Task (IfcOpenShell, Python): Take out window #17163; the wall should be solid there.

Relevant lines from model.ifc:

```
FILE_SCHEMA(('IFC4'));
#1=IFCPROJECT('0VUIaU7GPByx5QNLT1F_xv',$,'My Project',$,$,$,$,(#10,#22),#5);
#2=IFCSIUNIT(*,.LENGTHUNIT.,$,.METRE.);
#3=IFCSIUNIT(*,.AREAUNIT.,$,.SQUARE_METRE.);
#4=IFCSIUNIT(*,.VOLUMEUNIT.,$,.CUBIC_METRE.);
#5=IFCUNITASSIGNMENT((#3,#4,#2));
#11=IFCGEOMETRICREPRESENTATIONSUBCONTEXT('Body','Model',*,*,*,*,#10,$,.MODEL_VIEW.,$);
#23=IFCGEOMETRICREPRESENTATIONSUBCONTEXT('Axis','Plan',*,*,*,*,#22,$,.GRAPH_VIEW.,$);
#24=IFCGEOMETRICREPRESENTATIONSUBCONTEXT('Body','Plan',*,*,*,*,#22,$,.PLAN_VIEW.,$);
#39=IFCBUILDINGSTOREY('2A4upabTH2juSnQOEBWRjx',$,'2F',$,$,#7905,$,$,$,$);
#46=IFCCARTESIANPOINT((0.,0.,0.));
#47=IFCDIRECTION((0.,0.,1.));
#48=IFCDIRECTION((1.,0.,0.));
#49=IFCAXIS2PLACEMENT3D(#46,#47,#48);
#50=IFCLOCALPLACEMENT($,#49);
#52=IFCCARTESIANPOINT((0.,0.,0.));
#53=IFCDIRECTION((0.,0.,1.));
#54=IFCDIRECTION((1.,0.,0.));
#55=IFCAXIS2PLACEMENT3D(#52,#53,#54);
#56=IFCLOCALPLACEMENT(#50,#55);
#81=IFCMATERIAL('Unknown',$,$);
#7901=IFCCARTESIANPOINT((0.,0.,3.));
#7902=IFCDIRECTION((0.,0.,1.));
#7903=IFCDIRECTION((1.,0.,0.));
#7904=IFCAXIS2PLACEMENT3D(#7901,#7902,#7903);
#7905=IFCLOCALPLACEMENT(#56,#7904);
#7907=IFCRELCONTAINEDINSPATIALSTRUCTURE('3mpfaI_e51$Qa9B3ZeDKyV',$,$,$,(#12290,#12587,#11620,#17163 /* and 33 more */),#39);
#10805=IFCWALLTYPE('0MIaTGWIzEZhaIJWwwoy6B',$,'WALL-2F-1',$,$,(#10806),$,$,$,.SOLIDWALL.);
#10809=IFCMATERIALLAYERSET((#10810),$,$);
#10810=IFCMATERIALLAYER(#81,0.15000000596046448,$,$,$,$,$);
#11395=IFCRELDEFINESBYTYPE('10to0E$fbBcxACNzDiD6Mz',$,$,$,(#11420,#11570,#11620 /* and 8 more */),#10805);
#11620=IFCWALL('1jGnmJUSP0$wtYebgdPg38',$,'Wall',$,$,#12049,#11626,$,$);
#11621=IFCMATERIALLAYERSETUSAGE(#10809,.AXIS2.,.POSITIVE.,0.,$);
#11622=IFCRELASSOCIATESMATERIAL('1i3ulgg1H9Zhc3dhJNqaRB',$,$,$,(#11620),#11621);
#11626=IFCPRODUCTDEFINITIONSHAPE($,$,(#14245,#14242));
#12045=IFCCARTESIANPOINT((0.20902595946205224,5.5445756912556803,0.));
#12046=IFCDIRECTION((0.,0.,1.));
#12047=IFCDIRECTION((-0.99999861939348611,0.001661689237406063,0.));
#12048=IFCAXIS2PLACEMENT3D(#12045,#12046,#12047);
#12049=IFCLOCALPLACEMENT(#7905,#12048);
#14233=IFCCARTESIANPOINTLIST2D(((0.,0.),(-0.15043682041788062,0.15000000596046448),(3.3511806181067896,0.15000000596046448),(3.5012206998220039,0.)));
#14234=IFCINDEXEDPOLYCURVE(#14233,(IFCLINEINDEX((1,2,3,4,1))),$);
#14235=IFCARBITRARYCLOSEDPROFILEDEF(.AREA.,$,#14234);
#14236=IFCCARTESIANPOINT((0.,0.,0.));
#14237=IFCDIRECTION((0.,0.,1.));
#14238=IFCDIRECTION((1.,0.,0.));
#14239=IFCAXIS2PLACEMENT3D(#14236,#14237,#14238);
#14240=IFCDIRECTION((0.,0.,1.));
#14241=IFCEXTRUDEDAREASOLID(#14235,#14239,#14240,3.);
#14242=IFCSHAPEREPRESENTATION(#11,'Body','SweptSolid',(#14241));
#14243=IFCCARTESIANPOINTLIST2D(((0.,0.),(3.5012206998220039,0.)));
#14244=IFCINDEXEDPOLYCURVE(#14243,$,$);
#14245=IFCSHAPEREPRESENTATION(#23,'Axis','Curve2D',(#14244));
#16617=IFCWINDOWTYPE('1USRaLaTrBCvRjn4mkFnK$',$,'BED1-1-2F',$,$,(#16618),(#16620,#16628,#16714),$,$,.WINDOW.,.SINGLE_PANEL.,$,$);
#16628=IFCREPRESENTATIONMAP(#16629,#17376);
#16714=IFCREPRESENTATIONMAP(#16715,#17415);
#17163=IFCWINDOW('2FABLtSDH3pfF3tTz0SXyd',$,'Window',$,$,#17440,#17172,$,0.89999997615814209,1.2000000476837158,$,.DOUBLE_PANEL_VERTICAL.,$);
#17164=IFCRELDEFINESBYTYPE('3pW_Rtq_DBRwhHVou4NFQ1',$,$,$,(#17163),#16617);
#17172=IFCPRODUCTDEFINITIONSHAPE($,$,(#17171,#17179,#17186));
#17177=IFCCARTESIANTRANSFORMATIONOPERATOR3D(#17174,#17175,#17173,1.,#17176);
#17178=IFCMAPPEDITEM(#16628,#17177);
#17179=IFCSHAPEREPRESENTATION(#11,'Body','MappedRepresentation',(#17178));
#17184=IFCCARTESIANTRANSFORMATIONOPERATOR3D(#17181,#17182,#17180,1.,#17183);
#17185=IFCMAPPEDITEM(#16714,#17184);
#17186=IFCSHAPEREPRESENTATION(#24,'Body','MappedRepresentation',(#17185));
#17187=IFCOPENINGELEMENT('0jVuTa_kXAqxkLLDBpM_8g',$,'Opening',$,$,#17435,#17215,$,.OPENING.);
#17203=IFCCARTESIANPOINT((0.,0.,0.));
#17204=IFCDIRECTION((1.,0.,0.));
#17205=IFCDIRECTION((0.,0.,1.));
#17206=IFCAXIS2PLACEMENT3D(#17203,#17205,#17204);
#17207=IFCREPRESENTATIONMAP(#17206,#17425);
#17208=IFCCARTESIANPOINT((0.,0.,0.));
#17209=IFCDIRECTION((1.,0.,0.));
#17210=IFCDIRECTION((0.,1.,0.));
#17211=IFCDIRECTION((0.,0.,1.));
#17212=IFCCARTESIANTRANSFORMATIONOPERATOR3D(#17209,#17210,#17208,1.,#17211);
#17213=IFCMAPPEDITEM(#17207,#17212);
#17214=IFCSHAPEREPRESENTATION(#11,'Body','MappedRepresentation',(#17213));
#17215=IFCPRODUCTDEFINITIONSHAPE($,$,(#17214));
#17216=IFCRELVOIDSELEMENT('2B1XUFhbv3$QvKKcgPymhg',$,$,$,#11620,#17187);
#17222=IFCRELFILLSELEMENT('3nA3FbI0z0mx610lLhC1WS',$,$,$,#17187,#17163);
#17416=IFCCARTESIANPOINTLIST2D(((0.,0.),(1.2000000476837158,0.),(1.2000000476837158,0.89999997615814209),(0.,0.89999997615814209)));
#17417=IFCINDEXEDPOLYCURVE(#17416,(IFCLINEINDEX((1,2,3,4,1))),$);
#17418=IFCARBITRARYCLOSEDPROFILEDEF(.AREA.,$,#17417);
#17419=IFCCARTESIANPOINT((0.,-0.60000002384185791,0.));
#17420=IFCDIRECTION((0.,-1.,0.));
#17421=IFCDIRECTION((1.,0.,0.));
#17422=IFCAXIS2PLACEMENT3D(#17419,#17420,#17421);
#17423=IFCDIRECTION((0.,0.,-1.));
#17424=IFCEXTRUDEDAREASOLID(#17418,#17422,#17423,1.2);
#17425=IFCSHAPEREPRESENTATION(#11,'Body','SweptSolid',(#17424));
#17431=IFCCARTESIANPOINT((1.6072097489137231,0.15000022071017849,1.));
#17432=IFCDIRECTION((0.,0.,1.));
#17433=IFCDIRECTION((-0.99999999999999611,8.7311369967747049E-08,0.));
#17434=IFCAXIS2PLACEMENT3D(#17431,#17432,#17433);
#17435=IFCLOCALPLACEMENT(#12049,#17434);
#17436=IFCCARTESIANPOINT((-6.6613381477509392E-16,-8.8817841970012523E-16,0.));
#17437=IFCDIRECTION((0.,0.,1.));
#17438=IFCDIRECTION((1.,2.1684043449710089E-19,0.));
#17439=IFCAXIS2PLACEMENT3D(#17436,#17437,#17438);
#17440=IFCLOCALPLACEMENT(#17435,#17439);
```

```python
import ifcopenshell
import ifcopenshell.api.feature
import ifcopenshell.api.root
import ifcopenshell.geom
import ifcopenshell.util.shape

model = ifcopenshell.open("model.ifc")
settings = ifcopenshell.geom.settings()


def volume(element):
    """Net volume in cubic metres, openings subtracted."""
    shape = ifcopenshell.geom.create_shape(settings, element)
    return ifcopenshell.util.shape.get_volume(shape.geometry)


window = model.by_guid("2FABLtSDH3pfF3tTz0SXyd")
opening = window.FillsVoids[0].RelatingOpeningElement
wall = opening.VoidsElements[0].RelatingBuildingElement
before = volume(wall)

ifcopenshell.api.root.remove_product(model, product=window)
ifcopenshell.api.feature.remove_feature(model, feature=opening)

after = volume(wall)

print(f"wall volume {before:.3f} -> {after:.3f} m3")

model.write("model_edited.ifc")
```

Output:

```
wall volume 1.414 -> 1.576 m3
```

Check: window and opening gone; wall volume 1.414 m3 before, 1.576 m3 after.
